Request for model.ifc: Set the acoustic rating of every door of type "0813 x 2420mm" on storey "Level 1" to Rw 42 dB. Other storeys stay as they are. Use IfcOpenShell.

First a look at what the model holds.

```python
import ifcopenshell
import ifcopenshell.util.element

model = ifcopenshell.open("model.ifc")
print(model.schema)
storey = next(s for s in model.by_type("IfcBuildingStorey") if s.Name == "Level 1")
doors = [e for e in ifcopenshell.util.element.get_decomposition(storey) if e.is_a("IfcDoor")]
seen = {}
for e in doors:
    element_type = ifcopenshell.util.element.get_type(e)
    key = (element_type.Name if element_type != e and element_type else None, ifcopenshell.util.element.get_pset(e, "Pset_DoorCommon", "AcousticRating"))
    seen[key] = seen.get(key, 0) + 1
for (name, value), count in sorted(seen.items(), key=str):
    print(count, "x", name, "|", value)
```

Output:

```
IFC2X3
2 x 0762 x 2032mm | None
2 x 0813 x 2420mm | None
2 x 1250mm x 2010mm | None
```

```python
import ifcopenshell
import ifcopenshell.api.pset
import ifcopenshell.util.element

model = ifcopenshell.open("model.ifc")

storey = next(s for s in model.by_type("IfcBuildingStorey") if s.Name == "Level 1")
doors = [e for e in ifcopenshell.util.element.get_decomposition(storey) if e.is_a("IfcDoor")]

count = 0
for e in doors:
    element_type = ifcopenshell.util.element.get_type(e)
    if element_type in (None, e) or element_type.Name != "0813 x 2420mm":
        continue
    # add_pset returns the element's existing set when there is one.
    pset = ifcopenshell.api.pset.add_pset(model, product=e, name="Pset_DoorCommon")
    ifcopenshell.api.pset.edit_pset(model, pset=pset, properties={"AcousticRating": "Rw 42 dB"})
    count += 1

print(count, "doors updated")

model.write("model_rev.ifc")
```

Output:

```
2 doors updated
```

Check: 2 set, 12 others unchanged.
